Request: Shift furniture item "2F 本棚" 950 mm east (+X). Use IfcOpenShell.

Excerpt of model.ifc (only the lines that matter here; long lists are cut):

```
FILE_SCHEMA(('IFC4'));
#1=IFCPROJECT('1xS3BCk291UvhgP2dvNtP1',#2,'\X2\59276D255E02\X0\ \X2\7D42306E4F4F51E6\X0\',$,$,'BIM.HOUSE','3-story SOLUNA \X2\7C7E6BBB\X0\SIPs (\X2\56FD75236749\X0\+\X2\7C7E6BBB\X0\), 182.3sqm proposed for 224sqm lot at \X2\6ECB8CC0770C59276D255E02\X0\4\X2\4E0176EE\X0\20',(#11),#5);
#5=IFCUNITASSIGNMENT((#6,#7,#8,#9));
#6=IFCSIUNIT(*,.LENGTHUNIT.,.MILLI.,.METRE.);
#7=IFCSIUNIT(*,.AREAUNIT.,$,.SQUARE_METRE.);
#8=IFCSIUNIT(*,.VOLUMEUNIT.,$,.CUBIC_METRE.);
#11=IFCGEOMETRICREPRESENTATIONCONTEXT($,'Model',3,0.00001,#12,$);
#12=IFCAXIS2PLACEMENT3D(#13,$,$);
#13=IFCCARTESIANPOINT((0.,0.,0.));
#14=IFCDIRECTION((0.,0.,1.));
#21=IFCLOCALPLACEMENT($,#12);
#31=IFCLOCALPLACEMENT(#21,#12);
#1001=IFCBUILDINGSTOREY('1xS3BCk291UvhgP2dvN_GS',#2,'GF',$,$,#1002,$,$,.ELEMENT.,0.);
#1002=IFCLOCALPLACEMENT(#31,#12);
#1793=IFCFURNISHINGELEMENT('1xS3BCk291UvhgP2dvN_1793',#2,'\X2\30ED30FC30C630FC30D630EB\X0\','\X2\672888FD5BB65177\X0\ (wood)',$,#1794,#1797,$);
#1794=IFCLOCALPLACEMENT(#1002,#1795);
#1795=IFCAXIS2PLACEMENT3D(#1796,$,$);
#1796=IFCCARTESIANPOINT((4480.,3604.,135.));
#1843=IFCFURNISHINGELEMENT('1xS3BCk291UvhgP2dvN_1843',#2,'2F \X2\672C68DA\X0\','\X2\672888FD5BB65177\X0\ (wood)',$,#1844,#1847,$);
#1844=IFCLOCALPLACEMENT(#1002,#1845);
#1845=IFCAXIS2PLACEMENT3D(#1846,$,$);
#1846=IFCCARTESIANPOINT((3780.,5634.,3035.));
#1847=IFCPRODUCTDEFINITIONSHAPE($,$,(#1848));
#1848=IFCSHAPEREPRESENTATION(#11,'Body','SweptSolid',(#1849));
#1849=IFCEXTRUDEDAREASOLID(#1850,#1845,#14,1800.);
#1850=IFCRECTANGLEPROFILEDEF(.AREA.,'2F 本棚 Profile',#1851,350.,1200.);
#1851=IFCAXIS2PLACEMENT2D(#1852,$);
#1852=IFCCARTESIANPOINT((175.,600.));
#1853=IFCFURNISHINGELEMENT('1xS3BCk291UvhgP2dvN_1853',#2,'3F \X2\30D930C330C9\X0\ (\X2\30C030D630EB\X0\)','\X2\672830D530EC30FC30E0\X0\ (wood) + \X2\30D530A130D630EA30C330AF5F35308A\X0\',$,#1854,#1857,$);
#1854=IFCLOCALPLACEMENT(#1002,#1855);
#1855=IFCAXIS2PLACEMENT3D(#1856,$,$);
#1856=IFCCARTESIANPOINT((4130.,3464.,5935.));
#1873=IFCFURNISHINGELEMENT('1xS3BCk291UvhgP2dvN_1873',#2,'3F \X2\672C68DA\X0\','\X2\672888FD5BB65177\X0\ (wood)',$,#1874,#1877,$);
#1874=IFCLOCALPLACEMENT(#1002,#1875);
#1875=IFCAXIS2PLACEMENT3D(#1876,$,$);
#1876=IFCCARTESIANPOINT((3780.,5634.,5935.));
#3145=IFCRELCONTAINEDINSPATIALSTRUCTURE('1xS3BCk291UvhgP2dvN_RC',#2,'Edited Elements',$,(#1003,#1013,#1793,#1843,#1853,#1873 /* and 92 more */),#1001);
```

```python
import ifcopenshell
import ifcopenshell.api.geometry
import ifcopenshell.util.placement
import ifcopenshell.util.unit

model = ifcopenshell.open("model.ifc")
unit_scale = ifcopenshell.util.unit.calculate_unit_scale(model)

item = model.by_guid("1xS3BCk291UvhgP2dvN_1843")
matrix = ifcopenshell.util.placement.get_local_placement(item.ObjectPlacement)
matrix[0, 3] += 0.95 / unit_scale
ifcopenshell.api.geometry.edit_object_placement(model, product=item, matrix=matrix, is_si=False)

print(ifcopenshell.util.placement.get_local_placement(item.ObjectPlacement).round(3) + 0.0)

model.write("model-out.ifc")
```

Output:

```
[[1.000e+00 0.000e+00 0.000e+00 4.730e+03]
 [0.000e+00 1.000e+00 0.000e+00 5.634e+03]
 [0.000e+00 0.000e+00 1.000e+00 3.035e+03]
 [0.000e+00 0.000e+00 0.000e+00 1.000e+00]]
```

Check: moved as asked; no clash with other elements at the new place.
